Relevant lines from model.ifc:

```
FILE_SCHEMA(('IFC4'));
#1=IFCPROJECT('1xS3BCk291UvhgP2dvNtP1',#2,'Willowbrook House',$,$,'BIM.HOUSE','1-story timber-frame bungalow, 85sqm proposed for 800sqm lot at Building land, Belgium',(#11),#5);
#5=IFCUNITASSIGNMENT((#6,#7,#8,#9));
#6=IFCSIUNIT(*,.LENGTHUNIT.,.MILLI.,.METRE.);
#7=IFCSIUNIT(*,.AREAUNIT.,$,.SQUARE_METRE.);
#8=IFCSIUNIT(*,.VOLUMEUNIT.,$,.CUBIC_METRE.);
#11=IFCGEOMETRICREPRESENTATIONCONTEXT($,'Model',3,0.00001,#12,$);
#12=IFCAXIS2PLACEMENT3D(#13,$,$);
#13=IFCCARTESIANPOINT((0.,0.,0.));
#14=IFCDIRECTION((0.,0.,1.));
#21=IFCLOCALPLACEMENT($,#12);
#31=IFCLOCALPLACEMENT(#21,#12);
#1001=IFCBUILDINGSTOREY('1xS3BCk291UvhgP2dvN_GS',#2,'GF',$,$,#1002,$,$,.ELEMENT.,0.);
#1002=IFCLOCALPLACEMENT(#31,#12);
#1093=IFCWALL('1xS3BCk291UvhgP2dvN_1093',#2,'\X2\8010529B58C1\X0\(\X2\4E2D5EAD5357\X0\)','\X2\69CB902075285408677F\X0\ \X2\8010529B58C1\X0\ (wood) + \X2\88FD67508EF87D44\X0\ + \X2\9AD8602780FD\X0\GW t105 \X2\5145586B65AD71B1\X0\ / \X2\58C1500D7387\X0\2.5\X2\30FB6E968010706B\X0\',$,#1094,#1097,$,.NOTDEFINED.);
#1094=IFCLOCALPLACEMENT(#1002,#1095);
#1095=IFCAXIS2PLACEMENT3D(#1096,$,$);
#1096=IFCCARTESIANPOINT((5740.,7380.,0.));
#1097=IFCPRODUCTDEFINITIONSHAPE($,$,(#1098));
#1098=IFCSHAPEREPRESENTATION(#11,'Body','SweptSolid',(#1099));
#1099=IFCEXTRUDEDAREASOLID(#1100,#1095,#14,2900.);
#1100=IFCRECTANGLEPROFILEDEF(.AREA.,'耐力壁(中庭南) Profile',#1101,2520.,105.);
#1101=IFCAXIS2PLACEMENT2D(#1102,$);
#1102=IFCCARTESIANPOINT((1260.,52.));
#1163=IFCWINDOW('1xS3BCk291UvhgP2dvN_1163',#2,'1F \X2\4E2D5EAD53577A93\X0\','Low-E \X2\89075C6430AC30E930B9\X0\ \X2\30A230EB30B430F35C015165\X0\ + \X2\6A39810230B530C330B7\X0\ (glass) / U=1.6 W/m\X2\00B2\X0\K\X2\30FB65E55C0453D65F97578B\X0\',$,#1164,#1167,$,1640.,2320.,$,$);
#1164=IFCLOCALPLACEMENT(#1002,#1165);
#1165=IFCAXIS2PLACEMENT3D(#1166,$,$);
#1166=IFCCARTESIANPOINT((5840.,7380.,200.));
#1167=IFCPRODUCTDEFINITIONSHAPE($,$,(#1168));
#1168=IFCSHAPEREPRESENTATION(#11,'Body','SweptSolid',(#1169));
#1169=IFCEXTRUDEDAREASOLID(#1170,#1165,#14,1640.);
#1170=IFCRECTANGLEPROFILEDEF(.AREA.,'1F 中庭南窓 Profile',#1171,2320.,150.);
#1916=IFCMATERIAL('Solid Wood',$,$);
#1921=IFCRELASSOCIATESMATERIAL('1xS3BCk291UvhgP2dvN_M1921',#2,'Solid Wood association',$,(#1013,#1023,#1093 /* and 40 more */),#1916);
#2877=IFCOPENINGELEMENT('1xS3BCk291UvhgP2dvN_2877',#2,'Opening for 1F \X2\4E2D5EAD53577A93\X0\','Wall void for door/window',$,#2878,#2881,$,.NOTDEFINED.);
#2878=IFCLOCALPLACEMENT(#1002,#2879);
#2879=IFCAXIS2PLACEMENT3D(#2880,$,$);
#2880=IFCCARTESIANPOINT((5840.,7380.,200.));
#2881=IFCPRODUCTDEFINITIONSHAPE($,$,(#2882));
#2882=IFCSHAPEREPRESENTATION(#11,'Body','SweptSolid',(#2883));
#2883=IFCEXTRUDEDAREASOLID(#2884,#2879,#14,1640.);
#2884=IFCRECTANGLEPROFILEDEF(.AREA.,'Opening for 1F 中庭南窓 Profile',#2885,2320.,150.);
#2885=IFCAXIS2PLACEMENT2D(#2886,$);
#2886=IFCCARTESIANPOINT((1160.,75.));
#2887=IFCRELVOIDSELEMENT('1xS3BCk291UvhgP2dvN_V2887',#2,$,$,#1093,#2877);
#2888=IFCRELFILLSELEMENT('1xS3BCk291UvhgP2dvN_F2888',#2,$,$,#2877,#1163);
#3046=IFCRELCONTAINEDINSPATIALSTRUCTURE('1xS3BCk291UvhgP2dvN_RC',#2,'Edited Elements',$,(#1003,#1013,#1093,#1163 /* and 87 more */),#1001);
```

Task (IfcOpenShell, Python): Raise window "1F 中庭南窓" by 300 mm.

```python
import numpy as np
import ifcopenshell
import ifcopenshell.api.geometry
import ifcopenshell.util.placement
import ifcopenshell.util.unit

model = ifcopenshell.open("model.ifc")
unit_scale = ifcopenshell.util.unit.calculate_unit_scale(model)

window = model.by_id(1163)
opening = window.FillsVoids[0].RelatingOpeningElement
dz = 300.0

shift = np.array([0.0, 0.0, dz])
# The window is not placed relative to its opening, so move both.
for product in (opening, window):
    matrix = ifcopenshell.util.placement.get_local_placement(product.ObjectPlacement)
    matrix[:3, 3] += shift
    ifcopenshell.api.geometry.edit_object_placement(model, product=product, matrix=matrix, is_si=False)

print(f"moved by {dz * unit_scale:+.3f} m")

model.write("model-out.ifc")
```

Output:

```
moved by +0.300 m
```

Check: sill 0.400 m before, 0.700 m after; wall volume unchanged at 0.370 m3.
